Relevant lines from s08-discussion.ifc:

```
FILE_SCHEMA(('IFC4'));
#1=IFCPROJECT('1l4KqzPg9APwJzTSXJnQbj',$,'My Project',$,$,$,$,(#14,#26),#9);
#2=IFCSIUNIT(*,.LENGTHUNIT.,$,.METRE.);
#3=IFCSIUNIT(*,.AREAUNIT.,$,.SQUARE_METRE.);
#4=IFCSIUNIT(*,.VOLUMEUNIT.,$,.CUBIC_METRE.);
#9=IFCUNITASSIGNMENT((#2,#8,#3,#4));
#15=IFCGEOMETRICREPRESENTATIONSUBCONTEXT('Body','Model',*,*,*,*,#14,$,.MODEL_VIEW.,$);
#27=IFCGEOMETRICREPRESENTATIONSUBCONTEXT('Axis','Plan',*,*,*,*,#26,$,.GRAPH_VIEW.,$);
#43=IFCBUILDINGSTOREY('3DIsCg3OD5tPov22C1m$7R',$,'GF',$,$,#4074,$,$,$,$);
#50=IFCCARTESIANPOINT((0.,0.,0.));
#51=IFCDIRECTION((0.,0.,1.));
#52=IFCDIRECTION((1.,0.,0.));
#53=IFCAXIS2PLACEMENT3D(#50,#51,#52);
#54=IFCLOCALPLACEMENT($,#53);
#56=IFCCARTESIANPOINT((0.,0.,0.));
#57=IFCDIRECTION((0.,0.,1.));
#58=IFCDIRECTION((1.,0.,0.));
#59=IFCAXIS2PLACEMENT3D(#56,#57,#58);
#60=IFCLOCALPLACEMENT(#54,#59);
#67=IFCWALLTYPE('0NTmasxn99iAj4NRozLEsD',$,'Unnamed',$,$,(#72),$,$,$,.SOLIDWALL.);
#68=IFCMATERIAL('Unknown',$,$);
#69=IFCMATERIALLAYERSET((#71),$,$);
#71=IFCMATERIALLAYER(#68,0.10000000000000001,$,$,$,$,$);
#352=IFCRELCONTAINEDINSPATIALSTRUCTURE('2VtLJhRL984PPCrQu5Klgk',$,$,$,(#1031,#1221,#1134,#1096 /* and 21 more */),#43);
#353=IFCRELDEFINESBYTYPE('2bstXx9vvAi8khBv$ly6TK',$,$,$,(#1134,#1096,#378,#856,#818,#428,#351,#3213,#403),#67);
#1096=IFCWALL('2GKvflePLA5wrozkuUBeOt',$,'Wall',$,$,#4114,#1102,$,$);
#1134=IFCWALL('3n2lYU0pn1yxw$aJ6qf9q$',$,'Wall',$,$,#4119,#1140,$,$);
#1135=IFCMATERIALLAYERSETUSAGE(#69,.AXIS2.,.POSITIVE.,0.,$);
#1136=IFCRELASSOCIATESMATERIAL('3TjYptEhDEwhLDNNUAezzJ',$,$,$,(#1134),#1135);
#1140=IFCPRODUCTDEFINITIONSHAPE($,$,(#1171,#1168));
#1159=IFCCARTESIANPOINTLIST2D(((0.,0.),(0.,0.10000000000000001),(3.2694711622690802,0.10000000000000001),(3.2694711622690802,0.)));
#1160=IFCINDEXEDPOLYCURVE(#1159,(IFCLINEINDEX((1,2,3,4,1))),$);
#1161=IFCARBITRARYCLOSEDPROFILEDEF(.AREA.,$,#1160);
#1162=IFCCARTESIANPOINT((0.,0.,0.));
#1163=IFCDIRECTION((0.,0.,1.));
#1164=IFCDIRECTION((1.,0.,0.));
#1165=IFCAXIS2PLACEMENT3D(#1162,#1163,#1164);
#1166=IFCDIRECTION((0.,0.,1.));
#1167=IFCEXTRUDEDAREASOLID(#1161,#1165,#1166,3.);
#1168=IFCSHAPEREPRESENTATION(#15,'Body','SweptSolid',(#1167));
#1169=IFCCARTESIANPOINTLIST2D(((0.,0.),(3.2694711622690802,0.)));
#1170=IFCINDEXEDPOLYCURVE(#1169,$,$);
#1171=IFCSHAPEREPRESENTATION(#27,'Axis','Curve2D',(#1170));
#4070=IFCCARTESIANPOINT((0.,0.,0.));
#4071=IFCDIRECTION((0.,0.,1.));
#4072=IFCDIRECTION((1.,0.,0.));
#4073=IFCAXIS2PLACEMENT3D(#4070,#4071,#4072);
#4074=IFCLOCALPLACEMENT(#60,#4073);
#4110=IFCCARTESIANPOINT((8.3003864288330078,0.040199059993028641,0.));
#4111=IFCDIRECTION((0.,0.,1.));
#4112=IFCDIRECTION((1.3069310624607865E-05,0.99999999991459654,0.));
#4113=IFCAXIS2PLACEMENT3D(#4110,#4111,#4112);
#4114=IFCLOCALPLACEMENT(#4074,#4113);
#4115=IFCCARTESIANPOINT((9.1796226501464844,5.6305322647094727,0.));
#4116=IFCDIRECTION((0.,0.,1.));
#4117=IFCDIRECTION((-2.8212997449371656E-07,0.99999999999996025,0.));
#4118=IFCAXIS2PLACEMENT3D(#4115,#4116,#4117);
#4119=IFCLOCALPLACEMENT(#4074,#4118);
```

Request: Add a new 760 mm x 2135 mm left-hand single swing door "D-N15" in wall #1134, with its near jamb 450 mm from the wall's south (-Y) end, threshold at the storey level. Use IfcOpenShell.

```python
import numpy as np
import ifcopenshell
import ifcopenshell.api.feature
import ifcopenshell.api.geometry
import ifcopenshell.api.root
import ifcopenshell.api.spatial
import ifcopenshell.geom
import ifcopenshell.util.element
import ifcopenshell.util.placement
import ifcopenshell.util.representation
import ifcopenshell.util.shape
import ifcopenshell.util.unit

model = ifcopenshell.open("s08-discussion.ifc")
unit_scale = ifcopenshell.util.unit.calculate_unit_scale(model)
settings = ifcopenshell.geom.settings()


def volume(element):
    """Net volume in cubic metres, openings subtracted."""
    shape = ifcopenshell.geom.create_shape(settings, element)
    return ifcopenshell.util.shape.get_volume(shape.geometry)


wall = model.by_guid("3n2lYU0pn1yxw$aJ6qf9q$")
storey = ifcopenshell.util.element.get_container(wall, ifc_class="IfcBuildingStorey")
context = ifcopenshell.util.representation.get_context(model, "Model", "Body", "MODEL_VIEW")
before = volume(wall)

width, height, from_end, sill = 0.76, 2.135, 0.45, 0.0  # metres

# The wall runs along its own X axis, and the end named is its -X end.
wall_shape = ifcopenshell.geom.create_shape(settings, wall)
x, y, z = ifcopenshell.util.shape.get_vertices(wall_shape.geometry).T
start = x.min() + from_end
face, thickness = float(y.min()), float(y.max() - y.min())
wall_matrix = ifcopenshell.util.placement.get_local_placement(wall.ObjectPlacement)
level = ifcopenshell.util.placement.get_local_placement(storey.ObjectPlacement)[2, 3]


def in_wall(x, y):
    """Placement at x, y metres in the wall's axes, at sill height."""
    matrix = wall_matrix.copy()
    matrix[:, 3] = wall_matrix @ np.array([x / unit_scale, y / unit_scale, 0.0, 1.0])
    matrix[2, 3] = level + sill / unit_scale
    return matrix


# Opening: a box that overshoots both wall faces by 50 mm.
opening = ifcopenshell.api.root.create_entity(model, ifc_class="IfcOpeningElement", predefined_type="OPENING")
box = ifcopenshell.api.geometry.add_wall_representation(
    model, context=context, length=width, height=height, thickness=thickness + 0.1
)
ifcopenshell.api.geometry.assign_representation(model, product=opening, representation=box)
ifcopenshell.api.geometry.edit_object_placement(model, product=opening, matrix=in_wall(start, face - 0.05), is_si=False)
ifcopenshell.api.feature.add_feature(model, feature=opening, element=wall)

door = ifcopenshell.api.root.create_entity(model, ifc_class="IfcDoor", name="D-N15", predefined_type="DOOR")
door.OverallWidth, door.OverallHeight = width / unit_scale, height / unit_scale
door.OperationType = "SINGLE_SWING_LEFT"
body = ifcopenshell.api.geometry.add_door_representation(
    model,
    context=context,
    overall_width=door.OverallWidth,
    overall_height=door.OverallHeight,
    operation_type="SINGLE_SWING_LEFT",
    lining_properties={"LiningDepth": thickness / unit_scale, "ThresholdDepth": thickness / unit_scale},
)
ifcopenshell.api.geometry.assign_representation(model, product=door, representation=body)
ifcopenshell.api.spatial.assign_container(model, products=[door], relating_structure=storey)
ifcopenshell.api.feature.add_filling(model, opening=opening, element=door)

# The lining spans the wall, so the door starts at the wall face.
ifcopenshell.api.geometry.edit_object_placement(model, product=door, matrix=in_wall(start, face), is_si=False)

after = volume(wall)

print(f"wall volume {before:.3f} -> {after:.3f} m3")

model.write("s08-discussion_updated.ifc")
```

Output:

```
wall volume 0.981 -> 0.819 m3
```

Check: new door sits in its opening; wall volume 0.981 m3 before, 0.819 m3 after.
